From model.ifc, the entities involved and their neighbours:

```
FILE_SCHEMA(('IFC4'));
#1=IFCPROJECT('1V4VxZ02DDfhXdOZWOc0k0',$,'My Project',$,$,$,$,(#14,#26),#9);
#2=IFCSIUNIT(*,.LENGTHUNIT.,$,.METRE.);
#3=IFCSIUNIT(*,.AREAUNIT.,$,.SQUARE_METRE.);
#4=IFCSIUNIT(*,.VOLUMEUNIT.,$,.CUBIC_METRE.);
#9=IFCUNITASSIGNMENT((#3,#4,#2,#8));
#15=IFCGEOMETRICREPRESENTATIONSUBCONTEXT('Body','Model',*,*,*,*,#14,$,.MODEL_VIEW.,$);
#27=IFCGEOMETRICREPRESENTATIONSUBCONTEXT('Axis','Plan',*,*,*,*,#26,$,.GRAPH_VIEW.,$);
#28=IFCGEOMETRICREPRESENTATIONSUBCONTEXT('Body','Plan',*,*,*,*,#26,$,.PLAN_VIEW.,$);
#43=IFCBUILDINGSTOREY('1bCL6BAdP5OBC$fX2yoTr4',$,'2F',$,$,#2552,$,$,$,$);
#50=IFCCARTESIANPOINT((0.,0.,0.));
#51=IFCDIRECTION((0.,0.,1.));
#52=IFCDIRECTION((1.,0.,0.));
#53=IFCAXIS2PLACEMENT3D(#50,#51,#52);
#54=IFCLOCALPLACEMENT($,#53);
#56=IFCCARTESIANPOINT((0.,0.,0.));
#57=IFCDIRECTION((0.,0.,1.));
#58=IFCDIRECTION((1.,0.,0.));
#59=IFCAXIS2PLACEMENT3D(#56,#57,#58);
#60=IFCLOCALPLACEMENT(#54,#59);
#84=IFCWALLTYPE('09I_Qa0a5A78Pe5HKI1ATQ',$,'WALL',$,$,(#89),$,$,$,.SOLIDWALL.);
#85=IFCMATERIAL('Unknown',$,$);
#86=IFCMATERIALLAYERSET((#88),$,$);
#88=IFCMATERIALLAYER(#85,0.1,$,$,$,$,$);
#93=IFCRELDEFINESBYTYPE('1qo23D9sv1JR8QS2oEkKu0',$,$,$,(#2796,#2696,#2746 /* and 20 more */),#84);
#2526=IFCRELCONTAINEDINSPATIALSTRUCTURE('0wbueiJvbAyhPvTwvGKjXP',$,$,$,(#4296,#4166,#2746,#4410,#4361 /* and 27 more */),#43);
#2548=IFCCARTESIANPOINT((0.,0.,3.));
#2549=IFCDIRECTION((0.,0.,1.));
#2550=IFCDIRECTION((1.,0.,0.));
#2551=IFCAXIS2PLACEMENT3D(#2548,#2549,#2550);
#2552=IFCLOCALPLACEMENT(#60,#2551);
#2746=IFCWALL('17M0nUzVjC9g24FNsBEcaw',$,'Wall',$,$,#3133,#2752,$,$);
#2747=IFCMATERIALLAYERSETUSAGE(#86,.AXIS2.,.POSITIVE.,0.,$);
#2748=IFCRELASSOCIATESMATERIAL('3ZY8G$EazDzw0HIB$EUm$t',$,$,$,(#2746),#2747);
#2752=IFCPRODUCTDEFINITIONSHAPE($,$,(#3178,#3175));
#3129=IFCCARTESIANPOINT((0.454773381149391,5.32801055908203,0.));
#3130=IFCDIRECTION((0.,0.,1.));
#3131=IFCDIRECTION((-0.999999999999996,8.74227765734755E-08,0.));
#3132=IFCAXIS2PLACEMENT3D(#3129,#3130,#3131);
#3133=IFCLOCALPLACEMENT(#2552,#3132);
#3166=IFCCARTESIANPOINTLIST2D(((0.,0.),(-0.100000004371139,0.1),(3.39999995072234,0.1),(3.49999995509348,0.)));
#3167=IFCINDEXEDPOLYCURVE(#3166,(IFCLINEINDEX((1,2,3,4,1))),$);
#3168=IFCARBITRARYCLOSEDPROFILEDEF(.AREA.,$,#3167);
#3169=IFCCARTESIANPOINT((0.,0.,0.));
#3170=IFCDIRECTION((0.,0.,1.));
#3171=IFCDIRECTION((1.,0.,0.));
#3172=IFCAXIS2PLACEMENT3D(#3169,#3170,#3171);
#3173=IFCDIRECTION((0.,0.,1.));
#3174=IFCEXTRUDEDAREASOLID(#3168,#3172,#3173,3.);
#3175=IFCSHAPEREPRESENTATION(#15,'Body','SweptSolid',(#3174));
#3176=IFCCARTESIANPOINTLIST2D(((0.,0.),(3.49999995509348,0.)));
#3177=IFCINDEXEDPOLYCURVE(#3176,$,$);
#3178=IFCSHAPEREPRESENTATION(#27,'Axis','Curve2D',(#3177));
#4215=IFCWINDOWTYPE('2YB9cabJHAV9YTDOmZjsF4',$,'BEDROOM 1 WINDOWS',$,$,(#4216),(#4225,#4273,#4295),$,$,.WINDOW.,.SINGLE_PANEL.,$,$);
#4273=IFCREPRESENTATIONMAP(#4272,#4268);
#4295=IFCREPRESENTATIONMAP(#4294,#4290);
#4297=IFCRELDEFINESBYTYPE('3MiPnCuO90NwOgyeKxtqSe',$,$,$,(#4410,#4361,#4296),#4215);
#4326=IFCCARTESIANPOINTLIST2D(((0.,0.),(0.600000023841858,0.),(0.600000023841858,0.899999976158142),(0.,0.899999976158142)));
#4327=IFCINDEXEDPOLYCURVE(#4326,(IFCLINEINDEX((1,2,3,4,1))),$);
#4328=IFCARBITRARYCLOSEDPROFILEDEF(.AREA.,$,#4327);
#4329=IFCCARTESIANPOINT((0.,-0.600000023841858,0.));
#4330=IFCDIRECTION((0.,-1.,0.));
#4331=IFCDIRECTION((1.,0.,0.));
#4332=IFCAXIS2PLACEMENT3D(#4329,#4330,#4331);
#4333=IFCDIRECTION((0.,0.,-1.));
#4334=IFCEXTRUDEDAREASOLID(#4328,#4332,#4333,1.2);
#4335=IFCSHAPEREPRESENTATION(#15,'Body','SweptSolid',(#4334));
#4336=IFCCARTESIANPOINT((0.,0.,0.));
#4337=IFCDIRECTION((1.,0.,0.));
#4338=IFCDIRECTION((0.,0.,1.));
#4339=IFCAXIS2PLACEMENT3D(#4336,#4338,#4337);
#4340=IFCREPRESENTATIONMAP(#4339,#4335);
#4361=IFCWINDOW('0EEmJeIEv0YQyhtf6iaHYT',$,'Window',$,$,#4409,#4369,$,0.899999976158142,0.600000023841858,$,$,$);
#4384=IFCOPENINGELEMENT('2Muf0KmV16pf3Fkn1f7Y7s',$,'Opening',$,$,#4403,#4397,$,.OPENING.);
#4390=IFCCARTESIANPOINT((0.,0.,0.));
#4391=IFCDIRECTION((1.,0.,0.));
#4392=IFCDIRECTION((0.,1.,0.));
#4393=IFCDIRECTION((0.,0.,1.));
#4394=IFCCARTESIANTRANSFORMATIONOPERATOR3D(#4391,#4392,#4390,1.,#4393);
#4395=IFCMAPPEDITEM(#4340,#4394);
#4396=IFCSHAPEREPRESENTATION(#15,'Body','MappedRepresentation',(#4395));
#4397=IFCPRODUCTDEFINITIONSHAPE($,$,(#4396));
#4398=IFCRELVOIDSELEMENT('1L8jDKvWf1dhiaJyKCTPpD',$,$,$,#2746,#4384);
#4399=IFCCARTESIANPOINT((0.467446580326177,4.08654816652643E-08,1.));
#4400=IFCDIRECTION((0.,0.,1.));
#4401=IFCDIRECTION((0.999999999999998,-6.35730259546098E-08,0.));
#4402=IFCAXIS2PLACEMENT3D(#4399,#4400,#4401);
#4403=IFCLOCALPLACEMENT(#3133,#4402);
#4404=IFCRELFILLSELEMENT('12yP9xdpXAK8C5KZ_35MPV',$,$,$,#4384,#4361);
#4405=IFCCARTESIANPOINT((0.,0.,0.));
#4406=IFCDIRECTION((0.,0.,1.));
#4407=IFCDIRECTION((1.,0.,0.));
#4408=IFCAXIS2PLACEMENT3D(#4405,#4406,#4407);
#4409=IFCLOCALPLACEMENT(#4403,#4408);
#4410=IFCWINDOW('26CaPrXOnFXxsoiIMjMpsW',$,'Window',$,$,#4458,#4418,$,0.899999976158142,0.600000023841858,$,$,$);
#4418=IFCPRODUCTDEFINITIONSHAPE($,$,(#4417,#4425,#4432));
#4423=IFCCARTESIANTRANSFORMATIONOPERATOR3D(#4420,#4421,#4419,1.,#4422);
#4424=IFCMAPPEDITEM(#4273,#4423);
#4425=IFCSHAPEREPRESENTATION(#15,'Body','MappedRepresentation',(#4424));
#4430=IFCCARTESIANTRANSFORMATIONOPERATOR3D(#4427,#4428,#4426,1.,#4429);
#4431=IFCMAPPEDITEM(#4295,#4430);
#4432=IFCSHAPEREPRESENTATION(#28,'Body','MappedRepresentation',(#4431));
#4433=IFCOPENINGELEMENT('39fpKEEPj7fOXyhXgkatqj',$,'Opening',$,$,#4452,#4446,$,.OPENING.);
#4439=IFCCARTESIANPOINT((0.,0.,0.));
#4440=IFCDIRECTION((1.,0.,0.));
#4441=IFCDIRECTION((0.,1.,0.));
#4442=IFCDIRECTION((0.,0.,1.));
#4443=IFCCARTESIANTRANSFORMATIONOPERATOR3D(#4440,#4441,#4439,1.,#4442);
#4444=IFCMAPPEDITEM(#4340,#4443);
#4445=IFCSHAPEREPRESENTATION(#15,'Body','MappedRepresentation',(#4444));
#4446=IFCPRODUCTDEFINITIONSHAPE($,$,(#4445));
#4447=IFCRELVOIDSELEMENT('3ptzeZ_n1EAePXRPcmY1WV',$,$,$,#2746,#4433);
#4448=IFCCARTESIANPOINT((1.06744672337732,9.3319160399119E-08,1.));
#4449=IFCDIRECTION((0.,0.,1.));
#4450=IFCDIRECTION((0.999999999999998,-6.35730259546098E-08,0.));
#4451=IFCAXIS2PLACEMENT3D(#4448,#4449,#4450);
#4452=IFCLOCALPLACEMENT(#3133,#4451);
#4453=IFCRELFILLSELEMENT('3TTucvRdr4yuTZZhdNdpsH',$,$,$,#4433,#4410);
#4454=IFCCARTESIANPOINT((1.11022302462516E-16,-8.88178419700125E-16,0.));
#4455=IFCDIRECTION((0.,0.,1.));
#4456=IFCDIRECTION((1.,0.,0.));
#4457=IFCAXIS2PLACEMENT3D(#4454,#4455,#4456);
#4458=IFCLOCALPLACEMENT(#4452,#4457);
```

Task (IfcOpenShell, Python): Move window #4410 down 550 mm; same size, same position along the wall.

```python
import numpy as np
import ifcopenshell
import ifcopenshell.api.geometry
import ifcopenshell.util.placement
import ifcopenshell.util.unit

model = ifcopenshell.open("model.ifc")
unit_scale = ifcopenshell.util.unit.calculate_unit_scale(model)

window = model.by_guid("26CaPrXOnFXxsoiIMjMpsW")
opening = window.FillsVoids[0].RelatingOpeningElement
dz = -0.55 / unit_scale

shift = np.array([0.0, 0.0, dz])
# The window is placed relative to its opening, so it follows when the opening moves.
matrix = ifcopenshell.util.placement.get_local_placement(opening.ObjectPlacement)
matrix[:3, 3] += shift
ifcopenshell.api.geometry.edit_object_placement(
    model, product=opening, matrix=matrix, is_si=False, should_transform_children=True
)

print(f"moved by {dz * unit_scale:+.3f} m")

model.write("model_edited.ifc")
```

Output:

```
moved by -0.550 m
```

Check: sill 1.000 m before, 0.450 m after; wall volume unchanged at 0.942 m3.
